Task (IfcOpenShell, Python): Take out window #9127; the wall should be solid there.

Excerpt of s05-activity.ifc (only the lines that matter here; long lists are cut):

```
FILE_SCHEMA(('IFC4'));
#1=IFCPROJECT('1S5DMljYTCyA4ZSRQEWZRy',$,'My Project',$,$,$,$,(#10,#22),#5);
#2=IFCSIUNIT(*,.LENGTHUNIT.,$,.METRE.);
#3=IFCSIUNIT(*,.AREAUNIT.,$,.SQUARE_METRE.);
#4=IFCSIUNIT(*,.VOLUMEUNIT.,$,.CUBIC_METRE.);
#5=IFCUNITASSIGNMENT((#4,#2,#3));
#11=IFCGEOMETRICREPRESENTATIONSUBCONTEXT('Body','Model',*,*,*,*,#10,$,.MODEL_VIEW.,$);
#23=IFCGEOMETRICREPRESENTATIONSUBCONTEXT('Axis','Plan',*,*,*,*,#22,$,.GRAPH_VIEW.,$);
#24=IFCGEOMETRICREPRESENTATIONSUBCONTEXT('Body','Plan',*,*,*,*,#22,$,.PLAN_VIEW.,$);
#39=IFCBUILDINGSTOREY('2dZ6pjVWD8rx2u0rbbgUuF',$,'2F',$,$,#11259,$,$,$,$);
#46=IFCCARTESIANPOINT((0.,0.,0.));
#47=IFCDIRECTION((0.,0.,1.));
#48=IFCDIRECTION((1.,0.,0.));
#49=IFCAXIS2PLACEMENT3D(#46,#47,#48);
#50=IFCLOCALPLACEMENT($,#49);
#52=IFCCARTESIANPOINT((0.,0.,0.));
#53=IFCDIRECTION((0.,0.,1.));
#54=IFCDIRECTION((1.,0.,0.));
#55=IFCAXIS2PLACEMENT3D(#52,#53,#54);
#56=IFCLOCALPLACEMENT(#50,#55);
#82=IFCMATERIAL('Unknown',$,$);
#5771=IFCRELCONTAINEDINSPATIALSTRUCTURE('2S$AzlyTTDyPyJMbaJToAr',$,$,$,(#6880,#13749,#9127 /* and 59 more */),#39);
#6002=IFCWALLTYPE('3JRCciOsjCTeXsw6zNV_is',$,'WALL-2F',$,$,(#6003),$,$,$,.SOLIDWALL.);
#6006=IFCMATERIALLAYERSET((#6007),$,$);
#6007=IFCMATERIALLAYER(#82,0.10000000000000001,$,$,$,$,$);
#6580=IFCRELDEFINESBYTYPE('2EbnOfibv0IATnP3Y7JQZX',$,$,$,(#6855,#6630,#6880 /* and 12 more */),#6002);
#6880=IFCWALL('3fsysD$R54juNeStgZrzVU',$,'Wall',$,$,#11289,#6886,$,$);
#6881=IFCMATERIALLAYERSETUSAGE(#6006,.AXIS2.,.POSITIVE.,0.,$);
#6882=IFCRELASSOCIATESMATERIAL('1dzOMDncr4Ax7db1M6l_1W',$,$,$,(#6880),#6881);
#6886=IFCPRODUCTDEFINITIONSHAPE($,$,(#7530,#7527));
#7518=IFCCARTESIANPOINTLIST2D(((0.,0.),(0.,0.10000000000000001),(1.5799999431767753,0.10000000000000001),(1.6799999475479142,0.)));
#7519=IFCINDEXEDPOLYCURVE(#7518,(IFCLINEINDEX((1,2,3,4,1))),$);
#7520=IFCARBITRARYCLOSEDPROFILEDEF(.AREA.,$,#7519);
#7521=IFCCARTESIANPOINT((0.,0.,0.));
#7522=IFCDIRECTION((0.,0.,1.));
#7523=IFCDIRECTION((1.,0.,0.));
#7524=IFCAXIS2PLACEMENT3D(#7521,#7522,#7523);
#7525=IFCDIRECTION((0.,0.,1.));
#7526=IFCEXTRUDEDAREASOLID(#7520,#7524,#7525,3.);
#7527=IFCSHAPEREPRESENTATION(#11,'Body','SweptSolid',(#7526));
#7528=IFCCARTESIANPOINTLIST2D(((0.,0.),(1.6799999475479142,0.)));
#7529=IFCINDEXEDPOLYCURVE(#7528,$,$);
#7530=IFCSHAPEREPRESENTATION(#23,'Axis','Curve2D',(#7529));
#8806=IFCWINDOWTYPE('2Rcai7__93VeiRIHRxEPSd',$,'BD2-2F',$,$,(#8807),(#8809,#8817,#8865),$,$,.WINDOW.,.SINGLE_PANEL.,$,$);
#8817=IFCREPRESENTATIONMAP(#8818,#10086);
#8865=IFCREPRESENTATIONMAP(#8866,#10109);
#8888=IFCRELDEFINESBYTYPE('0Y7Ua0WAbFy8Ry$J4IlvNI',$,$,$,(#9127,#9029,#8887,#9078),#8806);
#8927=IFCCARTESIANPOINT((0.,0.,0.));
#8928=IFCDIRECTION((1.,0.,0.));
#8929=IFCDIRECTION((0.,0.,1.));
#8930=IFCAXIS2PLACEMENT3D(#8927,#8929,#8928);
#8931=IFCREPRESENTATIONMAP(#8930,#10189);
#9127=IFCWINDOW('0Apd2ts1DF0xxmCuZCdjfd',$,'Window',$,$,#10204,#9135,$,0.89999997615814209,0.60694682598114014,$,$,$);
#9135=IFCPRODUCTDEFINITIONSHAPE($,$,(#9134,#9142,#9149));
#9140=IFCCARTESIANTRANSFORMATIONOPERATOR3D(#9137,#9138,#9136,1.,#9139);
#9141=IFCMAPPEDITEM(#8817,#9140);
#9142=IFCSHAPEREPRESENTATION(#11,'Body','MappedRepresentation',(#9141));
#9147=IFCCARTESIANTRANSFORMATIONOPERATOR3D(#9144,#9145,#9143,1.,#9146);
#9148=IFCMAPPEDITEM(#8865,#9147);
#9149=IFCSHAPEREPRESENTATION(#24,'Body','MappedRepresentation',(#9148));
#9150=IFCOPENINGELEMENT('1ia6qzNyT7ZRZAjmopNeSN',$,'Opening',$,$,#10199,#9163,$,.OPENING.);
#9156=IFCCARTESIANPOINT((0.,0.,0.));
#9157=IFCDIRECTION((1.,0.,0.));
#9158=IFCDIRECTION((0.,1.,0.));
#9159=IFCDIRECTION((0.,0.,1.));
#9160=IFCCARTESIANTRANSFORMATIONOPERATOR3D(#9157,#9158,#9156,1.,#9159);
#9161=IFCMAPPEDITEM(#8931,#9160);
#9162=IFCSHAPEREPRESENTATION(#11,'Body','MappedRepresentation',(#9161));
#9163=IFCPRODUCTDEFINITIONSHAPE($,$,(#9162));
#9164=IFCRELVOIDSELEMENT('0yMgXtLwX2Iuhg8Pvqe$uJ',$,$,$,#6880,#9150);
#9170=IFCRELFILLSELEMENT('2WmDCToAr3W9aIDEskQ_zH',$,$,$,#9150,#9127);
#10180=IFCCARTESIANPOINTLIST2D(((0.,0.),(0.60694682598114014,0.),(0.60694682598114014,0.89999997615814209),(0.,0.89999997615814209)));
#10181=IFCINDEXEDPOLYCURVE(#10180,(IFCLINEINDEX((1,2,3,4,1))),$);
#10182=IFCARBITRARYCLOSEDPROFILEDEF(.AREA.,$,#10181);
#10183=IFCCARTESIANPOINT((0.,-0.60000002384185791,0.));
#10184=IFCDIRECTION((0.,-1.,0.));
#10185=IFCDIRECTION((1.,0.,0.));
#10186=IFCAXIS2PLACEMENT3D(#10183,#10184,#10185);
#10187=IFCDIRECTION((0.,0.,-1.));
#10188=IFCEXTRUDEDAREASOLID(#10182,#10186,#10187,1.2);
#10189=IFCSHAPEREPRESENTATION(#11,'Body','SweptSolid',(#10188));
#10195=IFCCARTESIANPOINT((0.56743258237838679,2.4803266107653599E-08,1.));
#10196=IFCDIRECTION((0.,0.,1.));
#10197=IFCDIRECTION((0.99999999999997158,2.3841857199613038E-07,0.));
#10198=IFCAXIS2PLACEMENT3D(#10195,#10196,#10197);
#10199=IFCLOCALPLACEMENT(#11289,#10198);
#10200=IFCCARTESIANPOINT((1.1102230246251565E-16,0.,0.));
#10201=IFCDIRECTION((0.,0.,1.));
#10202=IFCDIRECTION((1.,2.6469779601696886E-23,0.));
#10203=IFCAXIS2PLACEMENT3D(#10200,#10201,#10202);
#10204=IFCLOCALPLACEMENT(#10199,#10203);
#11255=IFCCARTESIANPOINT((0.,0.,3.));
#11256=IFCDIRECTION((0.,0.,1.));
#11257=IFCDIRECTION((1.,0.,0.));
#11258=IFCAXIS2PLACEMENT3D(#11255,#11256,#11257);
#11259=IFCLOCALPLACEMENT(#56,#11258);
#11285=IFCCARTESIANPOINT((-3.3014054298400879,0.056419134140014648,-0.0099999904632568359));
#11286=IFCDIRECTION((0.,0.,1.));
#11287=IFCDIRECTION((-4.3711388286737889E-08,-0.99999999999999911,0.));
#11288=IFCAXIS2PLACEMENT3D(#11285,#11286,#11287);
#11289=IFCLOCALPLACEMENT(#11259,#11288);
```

```python
import ifcopenshell
import ifcopenshell.api.feature
import ifcopenshell.api.root
import ifcopenshell.geom
import ifcopenshell.util.shape

model = ifcopenshell.open("s05-activity.ifc")
settings = ifcopenshell.geom.settings()


def volume(element):
    """Net volume in cubic metres, openings subtracted."""
    shape = ifcopenshell.geom.create_shape(settings, element)
    return ifcopenshell.util.shape.get_volume(shape.geometry)


window = model.by_guid("0Apd2ts1DF0xxmCuZCdjfd")
opening = window.FillsVoids[0].RelatingOpeningElement
wall = opening.VoidsElements[0].RelatingBuildingElement
before = volume(wall)

ifcopenshell.api.root.remove_product(model, product=window)
ifcopenshell.api.feature.remove_feature(model, feature=opening)

after = volume(wall)

print(f"wall volume {before:.3f} -> {after:.3f} m3")

model.write("s05-activity_rev.ifc")
```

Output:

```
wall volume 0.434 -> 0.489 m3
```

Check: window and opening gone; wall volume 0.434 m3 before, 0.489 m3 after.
